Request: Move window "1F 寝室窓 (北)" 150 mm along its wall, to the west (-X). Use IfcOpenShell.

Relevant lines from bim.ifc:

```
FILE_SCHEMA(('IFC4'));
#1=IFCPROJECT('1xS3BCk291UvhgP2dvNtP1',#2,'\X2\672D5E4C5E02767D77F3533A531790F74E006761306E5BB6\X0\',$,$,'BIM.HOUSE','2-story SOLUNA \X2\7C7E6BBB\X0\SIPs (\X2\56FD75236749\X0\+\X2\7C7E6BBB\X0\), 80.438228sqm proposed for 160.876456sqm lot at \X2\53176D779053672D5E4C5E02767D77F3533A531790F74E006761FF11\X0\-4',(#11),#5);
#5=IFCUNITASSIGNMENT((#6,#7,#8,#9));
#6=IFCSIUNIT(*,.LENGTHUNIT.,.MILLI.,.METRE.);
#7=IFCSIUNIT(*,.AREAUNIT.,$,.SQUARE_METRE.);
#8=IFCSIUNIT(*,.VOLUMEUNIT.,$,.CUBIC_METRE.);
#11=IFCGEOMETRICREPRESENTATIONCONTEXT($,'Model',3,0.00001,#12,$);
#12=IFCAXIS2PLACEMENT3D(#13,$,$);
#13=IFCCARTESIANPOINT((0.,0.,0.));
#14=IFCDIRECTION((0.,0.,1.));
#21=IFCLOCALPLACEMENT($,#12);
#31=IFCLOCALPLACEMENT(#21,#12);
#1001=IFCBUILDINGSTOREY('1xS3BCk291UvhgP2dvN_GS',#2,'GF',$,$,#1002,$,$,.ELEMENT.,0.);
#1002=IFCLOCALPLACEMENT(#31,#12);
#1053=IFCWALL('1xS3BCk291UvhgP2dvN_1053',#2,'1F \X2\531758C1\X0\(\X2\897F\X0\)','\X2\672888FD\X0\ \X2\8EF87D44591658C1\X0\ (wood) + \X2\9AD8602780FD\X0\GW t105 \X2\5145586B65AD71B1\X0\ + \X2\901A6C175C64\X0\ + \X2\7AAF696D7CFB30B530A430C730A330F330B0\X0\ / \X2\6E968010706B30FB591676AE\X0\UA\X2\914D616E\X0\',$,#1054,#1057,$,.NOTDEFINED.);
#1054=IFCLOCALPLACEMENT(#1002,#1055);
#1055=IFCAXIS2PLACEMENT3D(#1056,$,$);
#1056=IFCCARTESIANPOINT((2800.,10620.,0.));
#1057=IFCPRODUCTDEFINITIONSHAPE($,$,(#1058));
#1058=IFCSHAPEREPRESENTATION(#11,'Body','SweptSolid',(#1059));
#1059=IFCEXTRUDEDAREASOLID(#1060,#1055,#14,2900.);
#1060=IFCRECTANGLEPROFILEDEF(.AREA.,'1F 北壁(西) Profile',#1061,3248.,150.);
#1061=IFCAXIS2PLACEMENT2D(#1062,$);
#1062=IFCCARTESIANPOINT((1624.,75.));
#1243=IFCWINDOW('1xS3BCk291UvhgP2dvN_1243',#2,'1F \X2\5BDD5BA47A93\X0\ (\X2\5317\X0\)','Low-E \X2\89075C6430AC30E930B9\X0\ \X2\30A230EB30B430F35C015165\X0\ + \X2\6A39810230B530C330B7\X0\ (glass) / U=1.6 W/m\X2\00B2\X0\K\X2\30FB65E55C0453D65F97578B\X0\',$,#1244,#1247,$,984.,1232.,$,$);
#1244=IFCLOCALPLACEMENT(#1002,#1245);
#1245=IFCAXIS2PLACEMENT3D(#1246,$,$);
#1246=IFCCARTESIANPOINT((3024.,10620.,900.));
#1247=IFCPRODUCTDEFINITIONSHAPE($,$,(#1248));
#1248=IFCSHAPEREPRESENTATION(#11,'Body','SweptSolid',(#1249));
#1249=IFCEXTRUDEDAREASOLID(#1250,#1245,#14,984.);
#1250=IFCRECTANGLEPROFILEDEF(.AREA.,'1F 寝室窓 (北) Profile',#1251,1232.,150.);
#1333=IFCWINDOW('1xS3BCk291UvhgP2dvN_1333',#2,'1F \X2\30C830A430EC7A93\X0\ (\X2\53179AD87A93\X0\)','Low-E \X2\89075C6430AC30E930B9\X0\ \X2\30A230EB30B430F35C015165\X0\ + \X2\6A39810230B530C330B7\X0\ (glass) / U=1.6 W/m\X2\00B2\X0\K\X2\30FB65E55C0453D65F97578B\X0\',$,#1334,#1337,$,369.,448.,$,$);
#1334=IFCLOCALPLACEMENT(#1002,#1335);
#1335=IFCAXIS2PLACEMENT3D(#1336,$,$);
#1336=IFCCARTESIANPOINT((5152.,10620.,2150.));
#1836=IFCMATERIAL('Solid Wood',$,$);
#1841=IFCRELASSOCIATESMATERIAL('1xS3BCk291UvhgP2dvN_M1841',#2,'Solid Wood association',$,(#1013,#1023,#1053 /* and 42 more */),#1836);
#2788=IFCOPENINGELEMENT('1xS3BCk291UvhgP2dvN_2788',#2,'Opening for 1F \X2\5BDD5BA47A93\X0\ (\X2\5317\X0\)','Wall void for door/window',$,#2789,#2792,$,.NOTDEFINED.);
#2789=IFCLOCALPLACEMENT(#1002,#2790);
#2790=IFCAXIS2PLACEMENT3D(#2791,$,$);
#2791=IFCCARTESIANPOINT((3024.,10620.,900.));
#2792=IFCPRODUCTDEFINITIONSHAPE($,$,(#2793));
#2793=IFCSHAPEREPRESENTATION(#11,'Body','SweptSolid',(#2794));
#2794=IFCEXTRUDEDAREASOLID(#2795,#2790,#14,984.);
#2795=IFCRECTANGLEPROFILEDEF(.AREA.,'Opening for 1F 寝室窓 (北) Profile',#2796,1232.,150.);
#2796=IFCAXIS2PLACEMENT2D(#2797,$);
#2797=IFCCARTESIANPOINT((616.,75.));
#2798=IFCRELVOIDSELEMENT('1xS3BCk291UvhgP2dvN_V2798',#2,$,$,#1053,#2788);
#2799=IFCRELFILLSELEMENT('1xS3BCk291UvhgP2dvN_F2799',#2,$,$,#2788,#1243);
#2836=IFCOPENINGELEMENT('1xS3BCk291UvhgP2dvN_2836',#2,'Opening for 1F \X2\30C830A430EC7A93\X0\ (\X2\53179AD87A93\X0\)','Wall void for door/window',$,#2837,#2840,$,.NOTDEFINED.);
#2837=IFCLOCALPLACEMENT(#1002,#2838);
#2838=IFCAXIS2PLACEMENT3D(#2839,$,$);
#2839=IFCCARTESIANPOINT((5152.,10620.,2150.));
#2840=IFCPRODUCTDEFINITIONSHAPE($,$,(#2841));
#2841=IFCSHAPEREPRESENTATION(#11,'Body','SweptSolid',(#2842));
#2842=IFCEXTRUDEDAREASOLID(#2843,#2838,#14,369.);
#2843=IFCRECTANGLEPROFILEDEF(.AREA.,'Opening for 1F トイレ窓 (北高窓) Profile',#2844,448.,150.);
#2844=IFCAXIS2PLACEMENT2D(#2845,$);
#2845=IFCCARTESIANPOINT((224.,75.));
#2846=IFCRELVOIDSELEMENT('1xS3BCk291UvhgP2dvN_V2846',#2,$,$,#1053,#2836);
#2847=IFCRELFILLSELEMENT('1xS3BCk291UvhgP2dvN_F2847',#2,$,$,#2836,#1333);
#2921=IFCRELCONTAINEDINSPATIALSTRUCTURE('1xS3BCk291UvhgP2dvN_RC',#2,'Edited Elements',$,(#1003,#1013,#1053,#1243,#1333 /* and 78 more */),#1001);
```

```python
import ifcopenshell
import ifcopenshell.api.geometry
import ifcopenshell.util.placement
import ifcopenshell.util.unit

model = ifcopenshell.open("bim.ifc")
unit_scale = ifcopenshell.util.unit.calculate_unit_scale(model)

window = model.by_guid("1xS3BCk291UvhgP2dvN_1243")
opening = window.FillsVoids[0].RelatingOpeningElement
wall = opening.VoidsElements[0].RelatingBuildingElement

wall_matrix = ifcopenshell.util.placement.get_local_placement(wall.ObjectPlacement)
shift = wall_matrix[:3, 0] * -0.15 / unit_scale
before = ifcopenshell.util.placement.get_local_placement(window.ObjectPlacement)[:3, 3].copy()

# The window is not placed relative to its opening, so move both.
for product in (opening, window):
    matrix = ifcopenshell.util.placement.get_local_placement(product.ObjectPlacement)
    matrix[:3, 3] += shift
    ifcopenshell.api.geometry.edit_object_placement(model, product=product, matrix=matrix, is_si=False)

after = ifcopenshell.util.placement.get_local_placement(window.ObjectPlacement)[:3, 3]
print("window moved by", (after - before).round(3) + 0.0)

model.write("bim_rev.ifc")
```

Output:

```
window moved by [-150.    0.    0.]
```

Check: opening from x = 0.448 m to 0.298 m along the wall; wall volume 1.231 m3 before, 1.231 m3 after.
